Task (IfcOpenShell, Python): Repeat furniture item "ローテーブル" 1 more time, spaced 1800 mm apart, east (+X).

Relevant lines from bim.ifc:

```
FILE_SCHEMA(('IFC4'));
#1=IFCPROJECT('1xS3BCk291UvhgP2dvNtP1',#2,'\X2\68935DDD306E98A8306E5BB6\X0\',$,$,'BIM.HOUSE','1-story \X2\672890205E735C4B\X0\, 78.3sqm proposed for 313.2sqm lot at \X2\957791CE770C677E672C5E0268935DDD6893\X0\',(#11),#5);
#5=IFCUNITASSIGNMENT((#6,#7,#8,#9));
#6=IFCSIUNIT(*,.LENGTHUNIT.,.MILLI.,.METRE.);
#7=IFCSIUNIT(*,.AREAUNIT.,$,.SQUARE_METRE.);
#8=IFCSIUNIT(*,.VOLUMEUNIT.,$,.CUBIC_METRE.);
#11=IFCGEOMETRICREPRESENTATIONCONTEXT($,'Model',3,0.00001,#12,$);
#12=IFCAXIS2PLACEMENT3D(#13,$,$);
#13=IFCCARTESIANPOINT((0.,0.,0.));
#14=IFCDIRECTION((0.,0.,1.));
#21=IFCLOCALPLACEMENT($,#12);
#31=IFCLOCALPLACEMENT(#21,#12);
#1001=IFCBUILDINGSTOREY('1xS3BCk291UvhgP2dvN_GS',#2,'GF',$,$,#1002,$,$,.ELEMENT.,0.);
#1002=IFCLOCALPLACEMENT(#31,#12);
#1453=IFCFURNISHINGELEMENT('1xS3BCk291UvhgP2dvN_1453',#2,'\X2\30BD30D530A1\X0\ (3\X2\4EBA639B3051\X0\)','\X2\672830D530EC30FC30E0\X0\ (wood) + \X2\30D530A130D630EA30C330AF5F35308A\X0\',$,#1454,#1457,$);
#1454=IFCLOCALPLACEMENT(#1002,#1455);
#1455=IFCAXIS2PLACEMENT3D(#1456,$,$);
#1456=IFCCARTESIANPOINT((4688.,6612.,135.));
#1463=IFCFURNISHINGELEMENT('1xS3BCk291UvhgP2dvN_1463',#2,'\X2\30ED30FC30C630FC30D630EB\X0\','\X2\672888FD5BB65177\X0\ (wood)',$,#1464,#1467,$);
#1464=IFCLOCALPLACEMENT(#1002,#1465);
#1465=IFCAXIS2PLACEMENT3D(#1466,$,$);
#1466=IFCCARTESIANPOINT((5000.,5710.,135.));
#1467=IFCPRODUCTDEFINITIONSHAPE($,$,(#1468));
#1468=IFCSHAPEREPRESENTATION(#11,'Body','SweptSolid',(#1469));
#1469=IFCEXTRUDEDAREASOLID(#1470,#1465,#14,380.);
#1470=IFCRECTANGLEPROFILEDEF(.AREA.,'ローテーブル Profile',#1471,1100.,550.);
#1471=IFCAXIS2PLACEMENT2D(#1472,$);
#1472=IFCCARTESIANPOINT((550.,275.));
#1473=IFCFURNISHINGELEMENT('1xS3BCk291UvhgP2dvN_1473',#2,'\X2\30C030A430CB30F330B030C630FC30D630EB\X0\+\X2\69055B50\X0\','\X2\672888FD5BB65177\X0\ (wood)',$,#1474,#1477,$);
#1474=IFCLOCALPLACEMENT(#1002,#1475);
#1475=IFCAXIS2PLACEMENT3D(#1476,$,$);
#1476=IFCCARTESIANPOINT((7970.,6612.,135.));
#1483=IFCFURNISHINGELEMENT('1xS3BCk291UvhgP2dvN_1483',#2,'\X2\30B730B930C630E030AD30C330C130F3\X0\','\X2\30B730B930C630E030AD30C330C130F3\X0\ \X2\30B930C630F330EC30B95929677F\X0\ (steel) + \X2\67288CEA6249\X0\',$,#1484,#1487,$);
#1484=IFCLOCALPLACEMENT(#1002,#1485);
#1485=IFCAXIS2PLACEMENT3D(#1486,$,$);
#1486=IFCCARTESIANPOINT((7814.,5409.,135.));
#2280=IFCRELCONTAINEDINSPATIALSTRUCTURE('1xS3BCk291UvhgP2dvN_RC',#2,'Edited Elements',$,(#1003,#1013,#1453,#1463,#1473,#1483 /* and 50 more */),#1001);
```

```python
import numpy as np
import ifcopenshell
import ifcopenshell.api.geometry
import ifcopenshell.api.root
import ifcopenshell.util.element
import ifcopenshell.util.placement
import ifcopenshell.util.unit

model = ifcopenshell.open("bim.ifc")
unit_scale = ifcopenshell.util.unit.calculate_unit_scale(model)


def reuse_history(source, copy):
    """copy_class also copies each property set's owner history, people and application; keep the originals."""
    for rel in copy.IsDefinedBy:
        if rel.is_a("IfcRelDefinesByProperties") and (history := rel.RelatingPropertyDefinition.OwnerHistory):
            rel.RelatingPropertyDefinition.OwnerHistory = source.OwnerHistory
            ifcopenshell.util.element.remove_deep2(model, history)


source = model.by_id(1463)
base = ifcopenshell.util.placement.get_local_placement(source.ObjectPlacement)
step = np.array([1.0, 0.0, 0.0]) * 1.8 / unit_scale

for i in range(1, 2):
    copy = ifcopenshell.api.root.copy_class(model, product=source)
    copy.Representation = ifcopenshell.util.element.copy_deep(
        model, source.Representation, exclude=["IfcGeometricRepresentationContext", "IfcRepresentationMap"]
    )
    reuse_history(source, copy)
    matrix = base.copy()
    matrix[:3, 3] += i * step
    print("added at", matrix[:3, 3].round(3) + 0.0)
    ifcopenshell.api.geometry.edit_object_placement(model, product=copy, matrix=matrix, is_si=False)

model.write("bim-out.ifc")
```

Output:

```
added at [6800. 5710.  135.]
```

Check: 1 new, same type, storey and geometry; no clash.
